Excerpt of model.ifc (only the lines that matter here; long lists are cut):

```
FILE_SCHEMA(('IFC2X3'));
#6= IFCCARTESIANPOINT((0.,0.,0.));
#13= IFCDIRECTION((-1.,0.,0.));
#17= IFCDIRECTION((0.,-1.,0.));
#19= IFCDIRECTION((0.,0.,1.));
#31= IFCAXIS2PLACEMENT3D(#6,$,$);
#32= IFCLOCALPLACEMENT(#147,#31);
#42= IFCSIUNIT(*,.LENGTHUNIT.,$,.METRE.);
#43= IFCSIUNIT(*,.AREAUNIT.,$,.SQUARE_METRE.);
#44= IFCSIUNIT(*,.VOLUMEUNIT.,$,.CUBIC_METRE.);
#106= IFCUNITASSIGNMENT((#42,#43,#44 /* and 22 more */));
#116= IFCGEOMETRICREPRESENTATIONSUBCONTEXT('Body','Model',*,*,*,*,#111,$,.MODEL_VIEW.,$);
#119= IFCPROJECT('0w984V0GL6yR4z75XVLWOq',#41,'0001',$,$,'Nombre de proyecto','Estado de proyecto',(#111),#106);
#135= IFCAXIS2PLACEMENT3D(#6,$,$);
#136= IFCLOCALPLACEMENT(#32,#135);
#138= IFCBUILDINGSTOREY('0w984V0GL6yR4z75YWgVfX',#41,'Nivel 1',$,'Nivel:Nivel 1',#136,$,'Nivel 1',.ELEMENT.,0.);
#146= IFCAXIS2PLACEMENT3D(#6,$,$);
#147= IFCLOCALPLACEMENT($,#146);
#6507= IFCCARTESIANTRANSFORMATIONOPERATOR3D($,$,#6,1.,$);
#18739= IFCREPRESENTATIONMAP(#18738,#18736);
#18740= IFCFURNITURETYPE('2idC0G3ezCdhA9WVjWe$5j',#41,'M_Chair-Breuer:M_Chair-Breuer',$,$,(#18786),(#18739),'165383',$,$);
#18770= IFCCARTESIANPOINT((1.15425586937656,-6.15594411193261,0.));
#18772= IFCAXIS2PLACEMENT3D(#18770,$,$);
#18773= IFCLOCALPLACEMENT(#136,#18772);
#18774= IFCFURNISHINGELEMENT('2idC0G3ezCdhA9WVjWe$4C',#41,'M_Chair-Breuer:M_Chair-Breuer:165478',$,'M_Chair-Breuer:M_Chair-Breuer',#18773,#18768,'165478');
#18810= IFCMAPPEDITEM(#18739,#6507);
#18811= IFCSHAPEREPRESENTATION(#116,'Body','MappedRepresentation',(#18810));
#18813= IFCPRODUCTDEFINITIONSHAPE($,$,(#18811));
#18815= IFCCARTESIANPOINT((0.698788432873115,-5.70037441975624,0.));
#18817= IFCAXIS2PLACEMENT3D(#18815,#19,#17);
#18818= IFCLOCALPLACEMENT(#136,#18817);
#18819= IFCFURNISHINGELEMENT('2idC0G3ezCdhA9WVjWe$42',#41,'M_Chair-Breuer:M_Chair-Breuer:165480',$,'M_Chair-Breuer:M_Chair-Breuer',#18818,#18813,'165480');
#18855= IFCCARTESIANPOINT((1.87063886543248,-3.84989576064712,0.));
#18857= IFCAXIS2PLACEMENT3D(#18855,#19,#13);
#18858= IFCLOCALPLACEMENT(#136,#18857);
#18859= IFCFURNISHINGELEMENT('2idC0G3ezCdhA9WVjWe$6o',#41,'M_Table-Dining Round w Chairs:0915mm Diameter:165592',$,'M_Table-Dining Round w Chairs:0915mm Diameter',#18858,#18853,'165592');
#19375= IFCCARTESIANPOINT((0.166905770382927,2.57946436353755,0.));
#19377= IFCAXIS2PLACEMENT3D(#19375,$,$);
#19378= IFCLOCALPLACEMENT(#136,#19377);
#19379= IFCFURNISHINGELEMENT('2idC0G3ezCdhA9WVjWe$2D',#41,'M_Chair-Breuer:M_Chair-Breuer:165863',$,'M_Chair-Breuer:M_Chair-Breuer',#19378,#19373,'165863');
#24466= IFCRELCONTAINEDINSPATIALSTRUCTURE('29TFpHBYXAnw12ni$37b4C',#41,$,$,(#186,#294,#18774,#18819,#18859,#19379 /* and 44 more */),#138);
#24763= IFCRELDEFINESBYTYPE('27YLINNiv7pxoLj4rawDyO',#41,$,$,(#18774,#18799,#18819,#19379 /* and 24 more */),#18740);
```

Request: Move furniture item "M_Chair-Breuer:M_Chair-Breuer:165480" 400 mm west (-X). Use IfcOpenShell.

```python
import ifcopenshell
import ifcopenshell.api.geometry
import ifcopenshell.util.placement
import ifcopenshell.util.unit

model = ifcopenshell.open("model.ifc")
unit_scale = ifcopenshell.util.unit.calculate_unit_scale(model)

item = model.by_id(18819)
matrix = ifcopenshell.util.placement.get_local_placement(item.ObjectPlacement)
matrix[0, 3] -= 0.4 / unit_scale
ifcopenshell.api.geometry.edit_object_placement(model, product=item, matrix=matrix, is_si=False)

print(ifcopenshell.util.placement.get_local_placement(item.ObjectPlacement).round(3) + 0.0)

model.write("model_rev.ifc")
```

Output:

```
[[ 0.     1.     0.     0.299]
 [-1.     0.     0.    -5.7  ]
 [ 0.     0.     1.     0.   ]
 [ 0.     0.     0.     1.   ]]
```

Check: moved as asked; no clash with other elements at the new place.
